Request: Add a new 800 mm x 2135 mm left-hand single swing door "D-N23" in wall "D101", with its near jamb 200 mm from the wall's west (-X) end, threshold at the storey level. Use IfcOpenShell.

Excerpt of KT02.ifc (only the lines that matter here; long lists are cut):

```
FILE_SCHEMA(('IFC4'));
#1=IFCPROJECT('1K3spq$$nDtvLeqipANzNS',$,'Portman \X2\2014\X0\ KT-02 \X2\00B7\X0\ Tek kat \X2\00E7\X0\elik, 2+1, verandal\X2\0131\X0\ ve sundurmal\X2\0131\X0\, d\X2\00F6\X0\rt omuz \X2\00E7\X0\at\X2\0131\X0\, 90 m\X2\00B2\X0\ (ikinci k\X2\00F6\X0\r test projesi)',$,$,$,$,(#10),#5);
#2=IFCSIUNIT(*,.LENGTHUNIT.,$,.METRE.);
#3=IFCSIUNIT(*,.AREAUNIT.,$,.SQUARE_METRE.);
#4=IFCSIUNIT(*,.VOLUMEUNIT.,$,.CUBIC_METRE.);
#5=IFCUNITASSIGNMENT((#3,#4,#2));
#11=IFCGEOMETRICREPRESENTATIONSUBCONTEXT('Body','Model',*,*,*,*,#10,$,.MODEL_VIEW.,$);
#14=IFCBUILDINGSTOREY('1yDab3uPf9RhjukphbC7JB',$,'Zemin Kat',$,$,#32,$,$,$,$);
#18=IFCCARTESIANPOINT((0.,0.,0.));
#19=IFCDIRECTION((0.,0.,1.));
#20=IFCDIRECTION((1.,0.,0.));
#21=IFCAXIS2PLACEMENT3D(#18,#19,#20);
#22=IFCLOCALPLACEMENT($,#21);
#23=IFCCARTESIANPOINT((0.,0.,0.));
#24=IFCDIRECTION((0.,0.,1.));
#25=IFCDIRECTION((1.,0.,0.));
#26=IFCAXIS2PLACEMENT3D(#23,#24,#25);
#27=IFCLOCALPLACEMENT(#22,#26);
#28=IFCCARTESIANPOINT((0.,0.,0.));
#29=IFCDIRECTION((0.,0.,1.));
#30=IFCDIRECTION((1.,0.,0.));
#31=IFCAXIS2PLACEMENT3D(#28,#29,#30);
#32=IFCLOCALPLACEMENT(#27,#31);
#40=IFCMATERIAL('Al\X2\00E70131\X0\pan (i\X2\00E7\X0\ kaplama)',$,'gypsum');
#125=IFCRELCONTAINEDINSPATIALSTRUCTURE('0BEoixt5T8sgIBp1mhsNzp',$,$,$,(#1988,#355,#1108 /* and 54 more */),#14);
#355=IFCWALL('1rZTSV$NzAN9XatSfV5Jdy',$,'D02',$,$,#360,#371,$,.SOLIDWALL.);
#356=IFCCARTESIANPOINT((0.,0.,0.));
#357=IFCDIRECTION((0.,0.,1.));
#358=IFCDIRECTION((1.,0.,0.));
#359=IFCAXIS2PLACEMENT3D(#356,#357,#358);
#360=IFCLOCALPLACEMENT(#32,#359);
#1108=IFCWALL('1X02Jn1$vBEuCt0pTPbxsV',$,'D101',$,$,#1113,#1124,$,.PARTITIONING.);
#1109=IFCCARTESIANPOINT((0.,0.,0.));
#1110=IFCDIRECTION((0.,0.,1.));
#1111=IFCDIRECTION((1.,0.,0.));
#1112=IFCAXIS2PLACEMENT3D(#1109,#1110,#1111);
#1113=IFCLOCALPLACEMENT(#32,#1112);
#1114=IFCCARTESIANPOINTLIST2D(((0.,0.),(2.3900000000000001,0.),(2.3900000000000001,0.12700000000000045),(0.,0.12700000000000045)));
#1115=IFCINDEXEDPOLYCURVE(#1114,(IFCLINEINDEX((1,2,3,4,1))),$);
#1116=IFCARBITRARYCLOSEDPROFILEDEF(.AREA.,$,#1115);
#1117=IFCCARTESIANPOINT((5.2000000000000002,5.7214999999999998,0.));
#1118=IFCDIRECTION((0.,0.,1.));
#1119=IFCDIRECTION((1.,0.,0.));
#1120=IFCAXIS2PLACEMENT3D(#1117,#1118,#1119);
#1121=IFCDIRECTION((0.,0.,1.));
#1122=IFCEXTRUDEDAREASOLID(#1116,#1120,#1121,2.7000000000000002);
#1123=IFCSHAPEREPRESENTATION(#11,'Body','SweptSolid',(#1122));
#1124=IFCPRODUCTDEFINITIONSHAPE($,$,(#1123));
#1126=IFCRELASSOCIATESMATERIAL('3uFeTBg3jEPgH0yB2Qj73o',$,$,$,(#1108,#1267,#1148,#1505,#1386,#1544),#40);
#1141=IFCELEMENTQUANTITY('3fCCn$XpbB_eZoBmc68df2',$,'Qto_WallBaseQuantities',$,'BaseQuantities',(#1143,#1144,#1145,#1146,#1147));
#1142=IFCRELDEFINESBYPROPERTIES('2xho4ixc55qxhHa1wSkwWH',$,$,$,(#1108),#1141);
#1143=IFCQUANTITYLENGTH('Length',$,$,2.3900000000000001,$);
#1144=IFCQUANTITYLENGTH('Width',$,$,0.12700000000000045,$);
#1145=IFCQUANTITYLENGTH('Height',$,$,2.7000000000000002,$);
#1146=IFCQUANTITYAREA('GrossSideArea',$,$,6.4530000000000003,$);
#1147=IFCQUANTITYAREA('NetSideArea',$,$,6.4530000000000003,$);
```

```python
import numpy as np
import ifcopenshell
import ifcopenshell.api.feature
import ifcopenshell.api.geometry
import ifcopenshell.api.pset
import ifcopenshell.api.root
import ifcopenshell.api.spatial
import ifcopenshell.geom
import ifcopenshell.util.element
import ifcopenshell.util.placement
import ifcopenshell.util.representation
import ifcopenshell.util.shape
import ifcopenshell.util.unit

model = ifcopenshell.open("KT02.ifc")
unit_scale = ifcopenshell.util.unit.calculate_unit_scale(model)
area_scale = ifcopenshell.util.unit.calculate_unit_scale(model, "AREAUNIT")
settings = ifcopenshell.geom.settings()


def volume(element):
    """Net volume in cubic metres, openings subtracted."""
    shape = ifcopenshell.geom.create_shape(settings, element)
    return ifcopenshell.util.shape.get_volume(shape.geometry)


wall = model.by_id(1108)
storey = ifcopenshell.util.element.get_container(wall, ifc_class="IfcBuildingStorey")
context = ifcopenshell.util.representation.get_context(model, "Model", "Body", "MODEL_VIEW")
before = volume(wall)

width, height, from_end, sill = 0.8, 2.135, 0.2, 0.0  # metres

# The wall runs along its own X axis, and the end named is its -X end.
wall_shape = ifcopenshell.geom.create_shape(settings, wall)
x, y, z = ifcopenshell.util.shape.get_vertices(wall_shape.geometry).T
start = x.min() + from_end
face, thickness = float(y.min()), float(y.max() - y.min())
wall_matrix = ifcopenshell.util.placement.get_local_placement(wall.ObjectPlacement)
level = ifcopenshell.util.placement.get_local_placement(storey.ObjectPlacement)[2, 3]


def in_wall(x, y):
    """Placement at x, y metres in the wall's axes, at sill height."""
    matrix = wall_matrix.copy()
    matrix[:, 3] = wall_matrix @ np.array([x / unit_scale, y / unit_scale, 0.0, 1.0])
    matrix[2, 3] = level + sill / unit_scale
    return matrix


# Opening: a box that overshoots both wall faces by 50 mm.
opening = ifcopenshell.api.root.create_entity(model, ifc_class="IfcOpeningElement", predefined_type="OPENING")
box = ifcopenshell.api.geometry.add_wall_representation(
    model, context=context, length=width, height=height, thickness=thickness + 0.1
)
ifcopenshell.api.geometry.assign_representation(model, product=opening, representation=box)
ifcopenshell.api.geometry.edit_object_placement(model, product=opening, matrix=in_wall(start, face - 0.05), is_si=False)
ifcopenshell.api.feature.add_feature(model, feature=opening, element=wall)

door = ifcopenshell.api.root.create_entity(model, ifc_class="IfcDoor", name="D-N23", predefined_type="DOOR")
door.OverallWidth, door.OverallHeight = width / unit_scale, height / unit_scale
door.OperationType = "SINGLE_SWING_LEFT"
body = ifcopenshell.api.geometry.add_door_representation(
    model,
    context=context,
    overall_width=door.OverallWidth,
    overall_height=door.OverallHeight,
    operation_type="SINGLE_SWING_LEFT",
    lining_properties={"LiningDepth": thickness / unit_scale, "ThresholdDepth": thickness / unit_scale},
)
ifcopenshell.api.geometry.assign_representation(model, product=door, representation=body)
ifcopenshell.api.spatial.assign_container(model, products=[door], relating_structure=storey)
ifcopenshell.api.feature.add_filling(model, opening=opening, element=door)

# The lining spans the wall, so the door starts at the wall face.
ifcopenshell.api.geometry.edit_object_placement(model, product=door, matrix=in_wall(start, face), is_si=False)

after = volume(wall)

# Update the wall's stored quantities.
qto = model.by_id(ifcopenshell.util.element.get_pset(wall, "Qto_WallBaseQuantities", should_inherit=False)["id"])
ifcopenshell.api.pset.edit_qto(model, qto=qto, properties={"NetSideArea": after / thickness / area_scale})

print(f"wall volume {before:.3f} -> {after:.3f} m3")

model.write("KT02-out.ifc")
```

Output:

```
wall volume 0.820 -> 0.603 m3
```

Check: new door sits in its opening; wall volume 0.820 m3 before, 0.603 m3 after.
